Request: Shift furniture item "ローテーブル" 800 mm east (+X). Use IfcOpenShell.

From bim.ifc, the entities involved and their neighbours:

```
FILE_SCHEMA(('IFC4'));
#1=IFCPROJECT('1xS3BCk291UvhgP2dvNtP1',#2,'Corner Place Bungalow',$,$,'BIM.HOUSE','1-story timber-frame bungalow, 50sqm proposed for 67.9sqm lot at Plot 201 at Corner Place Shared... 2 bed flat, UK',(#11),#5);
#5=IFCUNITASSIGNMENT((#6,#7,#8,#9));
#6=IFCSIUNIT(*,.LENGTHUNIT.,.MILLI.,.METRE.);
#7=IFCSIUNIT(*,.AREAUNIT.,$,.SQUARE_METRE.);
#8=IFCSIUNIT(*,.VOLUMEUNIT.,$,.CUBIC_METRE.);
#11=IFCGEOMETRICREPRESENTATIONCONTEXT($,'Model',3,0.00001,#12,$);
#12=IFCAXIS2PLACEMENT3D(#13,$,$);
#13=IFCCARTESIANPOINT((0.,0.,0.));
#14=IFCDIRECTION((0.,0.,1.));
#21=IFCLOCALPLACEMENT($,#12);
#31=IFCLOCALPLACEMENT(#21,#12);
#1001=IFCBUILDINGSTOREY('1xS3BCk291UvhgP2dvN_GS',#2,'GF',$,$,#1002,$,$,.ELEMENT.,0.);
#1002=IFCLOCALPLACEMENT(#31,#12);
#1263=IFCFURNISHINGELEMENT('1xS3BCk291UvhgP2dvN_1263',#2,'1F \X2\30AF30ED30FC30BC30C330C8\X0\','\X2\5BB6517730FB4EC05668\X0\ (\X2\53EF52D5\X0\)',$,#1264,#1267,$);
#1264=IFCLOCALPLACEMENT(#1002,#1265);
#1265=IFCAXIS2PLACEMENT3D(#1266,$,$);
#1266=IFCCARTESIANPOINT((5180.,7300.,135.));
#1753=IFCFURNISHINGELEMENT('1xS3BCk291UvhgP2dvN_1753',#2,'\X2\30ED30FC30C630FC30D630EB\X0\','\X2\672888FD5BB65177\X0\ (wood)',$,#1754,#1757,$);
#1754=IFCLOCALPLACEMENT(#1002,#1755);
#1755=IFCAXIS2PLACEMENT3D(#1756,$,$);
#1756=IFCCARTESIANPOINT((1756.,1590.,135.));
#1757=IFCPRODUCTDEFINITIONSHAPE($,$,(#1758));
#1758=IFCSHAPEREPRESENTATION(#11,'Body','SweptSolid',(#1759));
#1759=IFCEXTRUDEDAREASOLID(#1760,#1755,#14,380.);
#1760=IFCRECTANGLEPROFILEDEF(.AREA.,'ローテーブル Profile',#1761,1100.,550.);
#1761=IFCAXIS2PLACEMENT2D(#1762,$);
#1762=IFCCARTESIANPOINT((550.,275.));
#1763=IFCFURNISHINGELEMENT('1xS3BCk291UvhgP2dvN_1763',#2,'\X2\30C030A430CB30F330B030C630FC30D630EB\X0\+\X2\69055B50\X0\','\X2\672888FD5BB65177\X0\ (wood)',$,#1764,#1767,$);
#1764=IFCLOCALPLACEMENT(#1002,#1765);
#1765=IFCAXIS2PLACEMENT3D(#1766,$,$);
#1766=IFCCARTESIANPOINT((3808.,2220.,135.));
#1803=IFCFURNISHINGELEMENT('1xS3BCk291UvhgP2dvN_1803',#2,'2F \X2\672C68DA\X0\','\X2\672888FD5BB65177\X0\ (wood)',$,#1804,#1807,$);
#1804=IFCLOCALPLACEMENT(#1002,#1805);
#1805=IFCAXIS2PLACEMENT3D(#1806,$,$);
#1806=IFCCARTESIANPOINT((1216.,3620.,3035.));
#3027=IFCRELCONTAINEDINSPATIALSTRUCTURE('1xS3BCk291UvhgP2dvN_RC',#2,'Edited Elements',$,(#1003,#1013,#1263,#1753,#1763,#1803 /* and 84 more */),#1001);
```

```python
import ifcopenshell
import ifcopenshell.api.geometry
import ifcopenshell.util.placement

model = ifcopenshell.open("bim.ifc")

item = model.by_guid("1xS3BCk291UvhgP2dvN_1753")
matrix = ifcopenshell.util.placement.get_local_placement(item.ObjectPlacement)
matrix[0, 3] += 800.0
ifcopenshell.api.geometry.edit_object_placement(model, product=item, matrix=matrix, is_si=False)

print(ifcopenshell.util.placement.get_local_placement(item.ObjectPlacement).round(3) + 0.0)

model.write("bim_v2.ifc")
```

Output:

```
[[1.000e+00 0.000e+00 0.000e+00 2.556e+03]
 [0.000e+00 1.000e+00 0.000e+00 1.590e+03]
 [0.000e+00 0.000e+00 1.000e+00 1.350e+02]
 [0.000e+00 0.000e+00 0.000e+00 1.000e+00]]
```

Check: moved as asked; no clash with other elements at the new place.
